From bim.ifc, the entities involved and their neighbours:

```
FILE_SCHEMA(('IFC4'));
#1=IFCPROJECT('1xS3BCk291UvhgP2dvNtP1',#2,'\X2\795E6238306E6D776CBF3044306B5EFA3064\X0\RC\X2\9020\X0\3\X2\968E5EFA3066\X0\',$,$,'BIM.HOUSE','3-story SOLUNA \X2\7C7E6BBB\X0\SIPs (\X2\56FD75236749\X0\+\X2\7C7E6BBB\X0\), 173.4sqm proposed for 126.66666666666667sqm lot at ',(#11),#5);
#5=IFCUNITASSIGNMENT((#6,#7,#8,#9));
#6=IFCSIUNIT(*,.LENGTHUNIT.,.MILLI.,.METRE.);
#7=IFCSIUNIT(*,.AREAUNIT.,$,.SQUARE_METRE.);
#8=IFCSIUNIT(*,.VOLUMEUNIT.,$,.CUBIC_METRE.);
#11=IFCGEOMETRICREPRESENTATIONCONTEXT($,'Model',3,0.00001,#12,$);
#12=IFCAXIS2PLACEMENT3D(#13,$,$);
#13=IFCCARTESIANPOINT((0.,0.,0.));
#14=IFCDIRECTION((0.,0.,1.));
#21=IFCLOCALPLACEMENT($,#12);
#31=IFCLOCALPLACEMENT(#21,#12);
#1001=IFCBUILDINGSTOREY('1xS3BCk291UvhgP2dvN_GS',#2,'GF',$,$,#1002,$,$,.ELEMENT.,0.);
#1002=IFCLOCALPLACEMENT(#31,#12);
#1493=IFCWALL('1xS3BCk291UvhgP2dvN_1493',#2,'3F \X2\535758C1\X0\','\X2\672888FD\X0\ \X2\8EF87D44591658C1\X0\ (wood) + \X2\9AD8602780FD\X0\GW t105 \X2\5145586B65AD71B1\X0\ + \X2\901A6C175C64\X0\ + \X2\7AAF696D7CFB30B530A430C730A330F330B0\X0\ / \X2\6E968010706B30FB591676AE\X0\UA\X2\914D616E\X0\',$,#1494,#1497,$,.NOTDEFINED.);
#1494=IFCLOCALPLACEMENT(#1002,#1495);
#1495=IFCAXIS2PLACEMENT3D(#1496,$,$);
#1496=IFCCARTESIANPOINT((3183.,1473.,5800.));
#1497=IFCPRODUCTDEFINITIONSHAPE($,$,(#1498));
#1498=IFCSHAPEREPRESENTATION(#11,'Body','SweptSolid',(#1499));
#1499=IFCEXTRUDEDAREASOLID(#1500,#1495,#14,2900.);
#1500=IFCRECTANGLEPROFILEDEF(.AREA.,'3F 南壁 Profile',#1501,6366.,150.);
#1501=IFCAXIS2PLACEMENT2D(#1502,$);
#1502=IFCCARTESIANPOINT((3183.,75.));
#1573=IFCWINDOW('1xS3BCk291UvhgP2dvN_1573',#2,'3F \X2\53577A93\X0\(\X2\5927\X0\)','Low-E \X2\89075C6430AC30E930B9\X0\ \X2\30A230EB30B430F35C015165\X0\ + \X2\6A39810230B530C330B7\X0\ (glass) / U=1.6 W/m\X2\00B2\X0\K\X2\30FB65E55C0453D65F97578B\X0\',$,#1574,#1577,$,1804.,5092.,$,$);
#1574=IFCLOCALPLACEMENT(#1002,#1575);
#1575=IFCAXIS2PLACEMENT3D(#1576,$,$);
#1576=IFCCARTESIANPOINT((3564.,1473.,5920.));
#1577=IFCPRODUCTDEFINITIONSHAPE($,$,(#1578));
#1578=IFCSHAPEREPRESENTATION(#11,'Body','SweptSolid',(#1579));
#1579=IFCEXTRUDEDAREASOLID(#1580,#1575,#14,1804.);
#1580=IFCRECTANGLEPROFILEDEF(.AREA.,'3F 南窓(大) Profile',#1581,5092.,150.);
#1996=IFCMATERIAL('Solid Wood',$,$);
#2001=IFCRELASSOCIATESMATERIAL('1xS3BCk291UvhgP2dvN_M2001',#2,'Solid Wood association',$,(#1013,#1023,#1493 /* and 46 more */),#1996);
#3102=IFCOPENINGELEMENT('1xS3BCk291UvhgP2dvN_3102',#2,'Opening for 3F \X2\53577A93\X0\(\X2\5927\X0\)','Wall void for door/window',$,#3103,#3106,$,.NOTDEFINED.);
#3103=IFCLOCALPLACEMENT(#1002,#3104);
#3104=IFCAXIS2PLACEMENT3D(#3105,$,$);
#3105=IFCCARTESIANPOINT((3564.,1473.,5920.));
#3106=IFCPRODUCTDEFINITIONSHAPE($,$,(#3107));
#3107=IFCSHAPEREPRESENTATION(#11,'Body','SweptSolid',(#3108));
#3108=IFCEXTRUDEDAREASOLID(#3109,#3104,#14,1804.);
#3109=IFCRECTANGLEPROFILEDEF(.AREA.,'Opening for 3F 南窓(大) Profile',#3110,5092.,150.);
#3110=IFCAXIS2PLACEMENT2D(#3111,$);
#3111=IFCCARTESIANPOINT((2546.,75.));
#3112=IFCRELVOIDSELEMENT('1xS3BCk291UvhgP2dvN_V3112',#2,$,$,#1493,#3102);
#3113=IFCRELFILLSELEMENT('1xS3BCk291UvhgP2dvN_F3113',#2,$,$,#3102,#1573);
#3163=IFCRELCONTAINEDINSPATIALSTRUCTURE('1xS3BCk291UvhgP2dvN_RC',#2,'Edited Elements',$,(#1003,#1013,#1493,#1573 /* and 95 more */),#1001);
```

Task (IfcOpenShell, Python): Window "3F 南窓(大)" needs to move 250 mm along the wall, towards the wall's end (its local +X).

```python
import ifcopenshell
import ifcopenshell.api.geometry
import ifcopenshell.util.placement
import ifcopenshell.util.unit

model = ifcopenshell.open("bim.ifc")
unit_scale = ifcopenshell.util.unit.calculate_unit_scale(model)

window = model.by_guid("1xS3BCk291UvhgP2dvN_1573")
opening = window.FillsVoids[0].RelatingOpeningElement
wall = opening.VoidsElements[0].RelatingBuildingElement

wall_matrix = ifcopenshell.util.placement.get_local_placement(wall.ObjectPlacement)
shift = wall_matrix[:3, 0] * 0.25 / unit_scale
before = ifcopenshell.util.placement.get_local_placement(window.ObjectPlacement)[:3, 3].copy()

# The window is not placed relative to its opening, so move both.
for product in (opening, window):
    matrix = ifcopenshell.util.placement.get_local_placement(product.ObjectPlacement)
    matrix[:3, 3] += shift
    ifcopenshell.api.geometry.edit_object_placement(model, product=product, matrix=matrix, is_si=False)

after = ifcopenshell.util.placement.get_local_placement(window.ObjectPlacement)[:3, 3]
print("window moved by", (after - before).round(3) + 0.0)

model.write("bim_rev.ifc")
```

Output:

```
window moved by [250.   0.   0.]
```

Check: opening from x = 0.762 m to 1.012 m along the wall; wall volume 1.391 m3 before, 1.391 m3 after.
